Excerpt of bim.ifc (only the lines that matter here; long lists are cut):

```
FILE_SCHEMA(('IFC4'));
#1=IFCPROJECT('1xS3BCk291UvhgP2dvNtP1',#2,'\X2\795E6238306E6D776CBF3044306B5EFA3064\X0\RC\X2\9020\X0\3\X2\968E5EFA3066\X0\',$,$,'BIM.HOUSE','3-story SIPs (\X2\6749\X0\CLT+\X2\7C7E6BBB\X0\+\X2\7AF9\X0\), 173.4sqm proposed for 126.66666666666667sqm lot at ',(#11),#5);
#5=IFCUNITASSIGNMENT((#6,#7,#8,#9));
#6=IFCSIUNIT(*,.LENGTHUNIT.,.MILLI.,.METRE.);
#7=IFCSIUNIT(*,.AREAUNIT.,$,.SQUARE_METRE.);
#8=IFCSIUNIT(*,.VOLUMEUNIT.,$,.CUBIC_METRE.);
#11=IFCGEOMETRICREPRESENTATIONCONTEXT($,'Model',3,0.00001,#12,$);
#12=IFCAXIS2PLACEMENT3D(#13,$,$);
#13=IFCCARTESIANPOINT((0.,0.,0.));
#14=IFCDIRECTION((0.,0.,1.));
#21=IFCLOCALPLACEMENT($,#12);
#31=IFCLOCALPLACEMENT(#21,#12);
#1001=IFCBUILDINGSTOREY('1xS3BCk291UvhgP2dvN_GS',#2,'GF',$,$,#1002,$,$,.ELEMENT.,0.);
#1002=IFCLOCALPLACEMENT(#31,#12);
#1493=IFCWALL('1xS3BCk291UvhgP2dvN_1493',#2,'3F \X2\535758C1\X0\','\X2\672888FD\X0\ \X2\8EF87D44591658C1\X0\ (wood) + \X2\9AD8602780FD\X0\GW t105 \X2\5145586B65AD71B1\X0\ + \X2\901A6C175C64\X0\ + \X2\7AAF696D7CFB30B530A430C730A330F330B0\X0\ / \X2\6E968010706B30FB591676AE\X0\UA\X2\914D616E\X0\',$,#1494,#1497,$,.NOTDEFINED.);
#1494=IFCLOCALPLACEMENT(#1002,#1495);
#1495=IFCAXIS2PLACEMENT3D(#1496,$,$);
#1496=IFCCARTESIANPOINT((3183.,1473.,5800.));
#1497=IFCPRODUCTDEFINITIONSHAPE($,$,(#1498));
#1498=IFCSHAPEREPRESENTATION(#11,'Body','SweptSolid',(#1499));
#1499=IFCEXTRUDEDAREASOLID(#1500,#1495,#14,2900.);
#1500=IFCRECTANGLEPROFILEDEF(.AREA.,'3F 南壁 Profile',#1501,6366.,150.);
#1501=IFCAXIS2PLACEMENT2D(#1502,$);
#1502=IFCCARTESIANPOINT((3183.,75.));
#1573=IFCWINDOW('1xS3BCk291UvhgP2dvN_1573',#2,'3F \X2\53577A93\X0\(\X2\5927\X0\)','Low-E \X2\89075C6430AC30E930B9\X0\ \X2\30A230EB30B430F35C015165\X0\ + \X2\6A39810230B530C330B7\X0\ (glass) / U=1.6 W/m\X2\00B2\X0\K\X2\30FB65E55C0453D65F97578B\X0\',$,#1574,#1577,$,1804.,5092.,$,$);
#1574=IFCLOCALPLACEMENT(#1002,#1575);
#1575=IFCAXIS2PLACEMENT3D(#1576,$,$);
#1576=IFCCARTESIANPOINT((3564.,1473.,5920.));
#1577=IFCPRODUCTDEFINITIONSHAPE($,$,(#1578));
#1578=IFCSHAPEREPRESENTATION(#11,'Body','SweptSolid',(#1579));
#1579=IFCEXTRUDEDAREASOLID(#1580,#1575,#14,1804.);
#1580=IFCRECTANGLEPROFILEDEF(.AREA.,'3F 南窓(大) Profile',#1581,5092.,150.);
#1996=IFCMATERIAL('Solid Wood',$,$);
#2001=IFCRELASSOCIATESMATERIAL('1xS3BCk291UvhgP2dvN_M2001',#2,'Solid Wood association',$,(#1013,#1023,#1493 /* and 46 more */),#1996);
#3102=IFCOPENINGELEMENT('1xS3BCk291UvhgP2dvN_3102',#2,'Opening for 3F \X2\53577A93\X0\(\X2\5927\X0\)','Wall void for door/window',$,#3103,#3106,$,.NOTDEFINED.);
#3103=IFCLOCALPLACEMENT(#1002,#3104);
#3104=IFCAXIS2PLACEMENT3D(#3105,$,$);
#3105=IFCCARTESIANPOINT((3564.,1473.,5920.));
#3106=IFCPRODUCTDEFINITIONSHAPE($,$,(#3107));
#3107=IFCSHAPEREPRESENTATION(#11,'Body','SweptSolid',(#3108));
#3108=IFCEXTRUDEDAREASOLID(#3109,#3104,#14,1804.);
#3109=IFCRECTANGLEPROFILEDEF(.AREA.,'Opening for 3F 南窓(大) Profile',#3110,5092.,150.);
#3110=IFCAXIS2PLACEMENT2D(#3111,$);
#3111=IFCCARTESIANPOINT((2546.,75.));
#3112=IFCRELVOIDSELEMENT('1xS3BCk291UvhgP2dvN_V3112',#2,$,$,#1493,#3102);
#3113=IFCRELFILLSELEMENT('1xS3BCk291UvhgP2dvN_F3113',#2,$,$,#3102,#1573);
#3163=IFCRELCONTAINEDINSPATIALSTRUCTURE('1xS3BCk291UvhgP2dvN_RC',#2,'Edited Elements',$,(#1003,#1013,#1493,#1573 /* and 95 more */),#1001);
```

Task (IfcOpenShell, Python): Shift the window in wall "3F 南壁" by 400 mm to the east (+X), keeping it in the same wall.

```python
import ifcopenshell
import ifcopenshell.api.geometry
import ifcopenshell.util.placement

model = ifcopenshell.open("bim.ifc")

window = model.by_guid("1xS3BCk291UvhgP2dvN_1573")
opening = window.FillsVoids[0].RelatingOpeningElement
wall = opening.VoidsElements[0].RelatingBuildingElement

wall_matrix = ifcopenshell.util.placement.get_local_placement(wall.ObjectPlacement)
shift = wall_matrix[:3, 0] * 400.0
before = ifcopenshell.util.placement.get_local_placement(window.ObjectPlacement)[:3, 3].copy()

# The window is not placed relative to its opening, so move both.
for product in (opening, window):
    matrix = ifcopenshell.util.placement.get_local_placement(product.ObjectPlacement)
    matrix[:3, 3] += shift
    ifcopenshell.api.geometry.edit_object_placement(model, product=product, matrix=matrix, is_si=False)

after = ifcopenshell.util.placement.get_local_placement(window.ObjectPlacement)[:3, 3]
print("window moved by", (after - before).round(3) + 0.0)

model.write("bim_updated.ifc")
```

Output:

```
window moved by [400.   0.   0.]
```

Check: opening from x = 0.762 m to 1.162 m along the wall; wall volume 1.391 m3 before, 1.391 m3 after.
